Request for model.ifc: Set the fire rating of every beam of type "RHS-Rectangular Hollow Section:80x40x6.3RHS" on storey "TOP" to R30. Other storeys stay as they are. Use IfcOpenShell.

First a look at what the model holds.

```python
import ifcopenshell
import ifcopenshell.util.element

model = ifcopenshell.open("model.ifc")
print(model.schema)
storey = next(s for s in model.by_type("IfcBuildingStorey") if s.Name == "TOP")
beams = [e for e in ifcopenshell.util.element.get_decomposition(storey) if e.is_a("IfcBeam")]
seen = {}
for e in beams:
    element_type = ifcopenshell.util.element.get_type(e)
    key = (element_type.Name if element_type != e and element_type else None, ifcopenshell.util.element.get_pset(e, "Pset_BeamCommon", "FireRating"))
    seen[key] = seen.get(key, 0) + 1
for (name, value), count in sorted(seen.items(), key=str):
    print(count, "x", name, "|", value)
```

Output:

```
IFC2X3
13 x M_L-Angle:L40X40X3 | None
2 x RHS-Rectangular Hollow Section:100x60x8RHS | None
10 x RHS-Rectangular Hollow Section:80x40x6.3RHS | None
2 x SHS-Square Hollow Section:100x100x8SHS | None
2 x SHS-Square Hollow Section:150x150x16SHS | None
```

```python
import ifcopenshell
import ifcopenshell.api.pset
import ifcopenshell.util.element

model = ifcopenshell.open("model.ifc")

storey = next(s for s in model.by_type("IfcBuildingStorey") if s.Name == "TOP")
beams = [e for e in ifcopenshell.util.element.get_decomposition(storey) if e.is_a("IfcBeam")]

count = 0
for e in beams:
    element_type = ifcopenshell.util.element.get_type(e)
    if element_type in (None, e) or element_type.Name != "RHS-Rectangular Hollow Section:80x40x6.3RHS":
        continue
    # add_pset returns the element's existing set when there is one.
    pset = ifcopenshell.api.pset.add_pset(model, product=e, name="Pset_BeamCommon")
    ifcopenshell.api.pset.edit_pset(model, pset=pset, properties={"FireRating": "R30"})
    count += 1

print(count, "beams updated")

model.write("model-out.ifc")
```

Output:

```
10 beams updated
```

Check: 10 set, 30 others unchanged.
